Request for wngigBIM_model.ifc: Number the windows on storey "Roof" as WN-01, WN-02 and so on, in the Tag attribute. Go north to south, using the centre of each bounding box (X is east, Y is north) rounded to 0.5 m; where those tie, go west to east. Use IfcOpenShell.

First a look at what the model holds.

```python
import ifcopenshell
import ifcopenshell.util.element
import ifcopenshell.util.placement

model = ifcopenshell.open("wngigBIM_model.ifc")
print(model.schema)
storey = next(s for s in model.by_type("IfcBuildingStorey") if s.Name == "Roof")
windows = [e for e in ifcopenshell.util.element.get_decomposition(storey) if e.is_a("IfcWindow")]
for e in sorted(windows, key=lambda e: e.id()):
    origin = ifcopenshell.util.placement.get_local_placement(e.ObjectPlacement)[:3, 3]
    print(e.id(), e.Tag, e.Name, origin.round(2) + 0.0, sep=" | ")
```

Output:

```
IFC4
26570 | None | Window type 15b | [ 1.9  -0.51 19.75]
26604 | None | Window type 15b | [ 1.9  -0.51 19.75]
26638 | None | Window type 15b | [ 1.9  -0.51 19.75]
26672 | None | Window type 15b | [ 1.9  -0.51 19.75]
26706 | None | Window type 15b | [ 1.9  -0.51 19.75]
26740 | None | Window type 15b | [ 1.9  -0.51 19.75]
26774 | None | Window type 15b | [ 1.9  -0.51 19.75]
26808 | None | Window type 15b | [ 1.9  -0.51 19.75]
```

```python
import ifcopenshell
import ifcopenshell.geom
import ifcopenshell.util.element
import ifcopenshell.util.shape

model = ifcopenshell.open("wngigBIM_model.ifc")
settings = ifcopenshell.geom.settings()
settings.set("use-world-coords", True)


def centre(element):
    shape = ifcopenshell.geom.create_shape(settings, element)
    return ifcopenshell.util.shape.get_bbox_centroid(shape.geometry)


storey = next(s for s in model.by_type("IfcBuildingStorey") if s.Name == "Roof")
windows = [e for e in ifcopenshell.util.element.get_decomposition(storey) if e.is_a("IfcWindow")]

# Insertion points can sit at a corner or the storey origin, so sort by the geometry (in metres).
centres = {e: centre(e) for e in windows}
windows.sort(key=lambda e: (-round(centres[e][1] / 0.5), centres[e][0]))

for i, e in enumerate(windows, start=1):
    number = f"WN-{i:02d}"
    e.Tag = number
    print(e.id(), number)

model.write("wngigBIM_model-out.ifc")
```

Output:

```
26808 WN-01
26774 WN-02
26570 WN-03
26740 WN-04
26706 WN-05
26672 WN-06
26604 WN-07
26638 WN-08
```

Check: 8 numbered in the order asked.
